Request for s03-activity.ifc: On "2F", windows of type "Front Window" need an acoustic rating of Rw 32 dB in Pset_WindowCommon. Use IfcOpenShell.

First a look at what the model holds.

```python
import ifcopenshell
import ifcopenshell.util.element

model = ifcopenshell.open("s03-activity.ifc")
print(model.schema)
storey = next(s for s in model.by_type("IfcBuildingStorey") if s.Name == "2F")
windows = [e for e in ifcopenshell.util.element.get_decomposition(storey) if e.is_a("IfcWindow")]
seen = {}
for e in windows:
    element_type = ifcopenshell.util.element.get_type(e)
    key = (element_type.Name if element_type != e and element_type else None, ifcopenshell.util.element.get_pset(e, "Pset_WindowCommon", "AcousticRating"))
    seen[key] = seen.get(key, 0) + 1
for (name, value), count in sorted(seen.items(), key=str):
    print(count, "x", name, "|", value)
```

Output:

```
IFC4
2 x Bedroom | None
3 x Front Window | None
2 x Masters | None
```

```python
import ifcopenshell
import ifcopenshell.api.pset
import ifcopenshell.util.element

model = ifcopenshell.open("s03-activity.ifc")

storey = next(s for s in model.by_type("IfcBuildingStorey") if s.Name == "2F")
windows = [e for e in ifcopenshell.util.element.get_decomposition(storey) if e.is_a("IfcWindow")]

count = 0
for e in windows:
    element_type = ifcopenshell.util.element.get_type(e)
    if element_type in (None, e) or element_type.Name != "Front Window":
        continue
    # add_pset returns the element's existing set when there is one.
    pset = ifcopenshell.api.pset.add_pset(model, product=e, name="Pset_WindowCommon")
    ifcopenshell.api.pset.edit_pset(model, pset=pset, properties={"AcousticRating": "Rw 32 dB"})
    count += 1

print(count, "windows updated")

model.write("s03-activity_edited.ifc")
```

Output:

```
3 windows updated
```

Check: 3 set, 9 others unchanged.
